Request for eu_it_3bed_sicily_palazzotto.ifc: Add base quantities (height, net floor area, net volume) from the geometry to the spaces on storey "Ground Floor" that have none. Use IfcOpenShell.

First a look at what the model holds.

```python
import ifcopenshell
import ifcopenshell.util.element
import ifcopenshell.util.unit

model = ifcopenshell.open("eu_it_3bed_sicily_palazzotto.ifc")
print(model.schema)
for unit_type in ("LENGTHUNIT", "AREAUNIT", "VOLUMEUNIT"):
    print(unit_type, ifcopenshell.util.unit.calculate_unit_scale(model, unit_type))
storey = next(s for s in model.by_type("IfcBuildingStorey") if s.Name == "Ground Floor")
spaces = [e for e in ifcopenshell.util.element.get_decomposition(storey) if e.is_a("IfcSpace")]
for e in sorted(spaces, key=lambda e: e.id()):
    print(e.id(), e.is_a(), e.Name, list(ifcopenshell.util.element.get_psets(e, qtos_only=True)), sep=" | ")
```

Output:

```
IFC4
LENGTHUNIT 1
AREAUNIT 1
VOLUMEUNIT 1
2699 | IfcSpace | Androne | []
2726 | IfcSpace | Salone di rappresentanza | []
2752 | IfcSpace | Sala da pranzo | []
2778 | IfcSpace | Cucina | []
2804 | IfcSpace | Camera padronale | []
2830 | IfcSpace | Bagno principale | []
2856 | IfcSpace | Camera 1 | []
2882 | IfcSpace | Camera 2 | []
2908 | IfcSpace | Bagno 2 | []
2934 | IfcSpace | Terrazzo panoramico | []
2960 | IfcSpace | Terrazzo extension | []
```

```python
import ifcopenshell
import ifcopenshell.api.pset
import ifcopenshell.geom
import ifcopenshell.util.element
import ifcopenshell.util.shape
import ifcopenshell.util.unit

model = ifcopenshell.open("eu_it_3bed_sicily_palazzotto.ifc")
unit_scale = ifcopenshell.util.unit.calculate_unit_scale(model)
area_scale = ifcopenshell.util.unit.calculate_unit_scale(model, "AREAUNIT")
volume_scale = ifcopenshell.util.unit.calculate_unit_scale(model, "VOLUMEUNIT")
settings = ifcopenshell.geom.settings()

storey = next(s for s in model.by_type("IfcBuildingStorey") if s.Name == "Ground Floor")
spaces = [e for e in ifcopenshell.util.element.get_decomposition(storey) if e.is_a("IfcSpace")]

for e in sorted(spaces, key=lambda e: e.id()):
    if ifcopenshell.util.element.get_psets(e, qtos_only=True, should_inherit=False):
        continue
    # Geometry comes back in metres, in the element's own axes.
    shape = ifcopenshell.geom.create_shape(settings, e)
    values = {
        "Height": ifcopenshell.util.shape.get_z(shape.geometry) / unit_scale,
        "NetFloorArea": ifcopenshell.util.shape.get_footprint_area(shape.geometry) / area_scale,
        "NetVolume": ifcopenshell.util.shape.get_volume(shape.geometry) / volume_scale,
    }
    qto = ifcopenshell.api.pset.add_qto(model, product=e, name="Qto_SpaceBaseQuantities")
    ifcopenshell.api.pset.edit_qto(model, qto=qto, properties=values)
    print(e.id(), {k: round(v, 3) for k, v in values.items()})

model.write("eu_it_3bed_sicily_palazzotto_edited.ifc")
```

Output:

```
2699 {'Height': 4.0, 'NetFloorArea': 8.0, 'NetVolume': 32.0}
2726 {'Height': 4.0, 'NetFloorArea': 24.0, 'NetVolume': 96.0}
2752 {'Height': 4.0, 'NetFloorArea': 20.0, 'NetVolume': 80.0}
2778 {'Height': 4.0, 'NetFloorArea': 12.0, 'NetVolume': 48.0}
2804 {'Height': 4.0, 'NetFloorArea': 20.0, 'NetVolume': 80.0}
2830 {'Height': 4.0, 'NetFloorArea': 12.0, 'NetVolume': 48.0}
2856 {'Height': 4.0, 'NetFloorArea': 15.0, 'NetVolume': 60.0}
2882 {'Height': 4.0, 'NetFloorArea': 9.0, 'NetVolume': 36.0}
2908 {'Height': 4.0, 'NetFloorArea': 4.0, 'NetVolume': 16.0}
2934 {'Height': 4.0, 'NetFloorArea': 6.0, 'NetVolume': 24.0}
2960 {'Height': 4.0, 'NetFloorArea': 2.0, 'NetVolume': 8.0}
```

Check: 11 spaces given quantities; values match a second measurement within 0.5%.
